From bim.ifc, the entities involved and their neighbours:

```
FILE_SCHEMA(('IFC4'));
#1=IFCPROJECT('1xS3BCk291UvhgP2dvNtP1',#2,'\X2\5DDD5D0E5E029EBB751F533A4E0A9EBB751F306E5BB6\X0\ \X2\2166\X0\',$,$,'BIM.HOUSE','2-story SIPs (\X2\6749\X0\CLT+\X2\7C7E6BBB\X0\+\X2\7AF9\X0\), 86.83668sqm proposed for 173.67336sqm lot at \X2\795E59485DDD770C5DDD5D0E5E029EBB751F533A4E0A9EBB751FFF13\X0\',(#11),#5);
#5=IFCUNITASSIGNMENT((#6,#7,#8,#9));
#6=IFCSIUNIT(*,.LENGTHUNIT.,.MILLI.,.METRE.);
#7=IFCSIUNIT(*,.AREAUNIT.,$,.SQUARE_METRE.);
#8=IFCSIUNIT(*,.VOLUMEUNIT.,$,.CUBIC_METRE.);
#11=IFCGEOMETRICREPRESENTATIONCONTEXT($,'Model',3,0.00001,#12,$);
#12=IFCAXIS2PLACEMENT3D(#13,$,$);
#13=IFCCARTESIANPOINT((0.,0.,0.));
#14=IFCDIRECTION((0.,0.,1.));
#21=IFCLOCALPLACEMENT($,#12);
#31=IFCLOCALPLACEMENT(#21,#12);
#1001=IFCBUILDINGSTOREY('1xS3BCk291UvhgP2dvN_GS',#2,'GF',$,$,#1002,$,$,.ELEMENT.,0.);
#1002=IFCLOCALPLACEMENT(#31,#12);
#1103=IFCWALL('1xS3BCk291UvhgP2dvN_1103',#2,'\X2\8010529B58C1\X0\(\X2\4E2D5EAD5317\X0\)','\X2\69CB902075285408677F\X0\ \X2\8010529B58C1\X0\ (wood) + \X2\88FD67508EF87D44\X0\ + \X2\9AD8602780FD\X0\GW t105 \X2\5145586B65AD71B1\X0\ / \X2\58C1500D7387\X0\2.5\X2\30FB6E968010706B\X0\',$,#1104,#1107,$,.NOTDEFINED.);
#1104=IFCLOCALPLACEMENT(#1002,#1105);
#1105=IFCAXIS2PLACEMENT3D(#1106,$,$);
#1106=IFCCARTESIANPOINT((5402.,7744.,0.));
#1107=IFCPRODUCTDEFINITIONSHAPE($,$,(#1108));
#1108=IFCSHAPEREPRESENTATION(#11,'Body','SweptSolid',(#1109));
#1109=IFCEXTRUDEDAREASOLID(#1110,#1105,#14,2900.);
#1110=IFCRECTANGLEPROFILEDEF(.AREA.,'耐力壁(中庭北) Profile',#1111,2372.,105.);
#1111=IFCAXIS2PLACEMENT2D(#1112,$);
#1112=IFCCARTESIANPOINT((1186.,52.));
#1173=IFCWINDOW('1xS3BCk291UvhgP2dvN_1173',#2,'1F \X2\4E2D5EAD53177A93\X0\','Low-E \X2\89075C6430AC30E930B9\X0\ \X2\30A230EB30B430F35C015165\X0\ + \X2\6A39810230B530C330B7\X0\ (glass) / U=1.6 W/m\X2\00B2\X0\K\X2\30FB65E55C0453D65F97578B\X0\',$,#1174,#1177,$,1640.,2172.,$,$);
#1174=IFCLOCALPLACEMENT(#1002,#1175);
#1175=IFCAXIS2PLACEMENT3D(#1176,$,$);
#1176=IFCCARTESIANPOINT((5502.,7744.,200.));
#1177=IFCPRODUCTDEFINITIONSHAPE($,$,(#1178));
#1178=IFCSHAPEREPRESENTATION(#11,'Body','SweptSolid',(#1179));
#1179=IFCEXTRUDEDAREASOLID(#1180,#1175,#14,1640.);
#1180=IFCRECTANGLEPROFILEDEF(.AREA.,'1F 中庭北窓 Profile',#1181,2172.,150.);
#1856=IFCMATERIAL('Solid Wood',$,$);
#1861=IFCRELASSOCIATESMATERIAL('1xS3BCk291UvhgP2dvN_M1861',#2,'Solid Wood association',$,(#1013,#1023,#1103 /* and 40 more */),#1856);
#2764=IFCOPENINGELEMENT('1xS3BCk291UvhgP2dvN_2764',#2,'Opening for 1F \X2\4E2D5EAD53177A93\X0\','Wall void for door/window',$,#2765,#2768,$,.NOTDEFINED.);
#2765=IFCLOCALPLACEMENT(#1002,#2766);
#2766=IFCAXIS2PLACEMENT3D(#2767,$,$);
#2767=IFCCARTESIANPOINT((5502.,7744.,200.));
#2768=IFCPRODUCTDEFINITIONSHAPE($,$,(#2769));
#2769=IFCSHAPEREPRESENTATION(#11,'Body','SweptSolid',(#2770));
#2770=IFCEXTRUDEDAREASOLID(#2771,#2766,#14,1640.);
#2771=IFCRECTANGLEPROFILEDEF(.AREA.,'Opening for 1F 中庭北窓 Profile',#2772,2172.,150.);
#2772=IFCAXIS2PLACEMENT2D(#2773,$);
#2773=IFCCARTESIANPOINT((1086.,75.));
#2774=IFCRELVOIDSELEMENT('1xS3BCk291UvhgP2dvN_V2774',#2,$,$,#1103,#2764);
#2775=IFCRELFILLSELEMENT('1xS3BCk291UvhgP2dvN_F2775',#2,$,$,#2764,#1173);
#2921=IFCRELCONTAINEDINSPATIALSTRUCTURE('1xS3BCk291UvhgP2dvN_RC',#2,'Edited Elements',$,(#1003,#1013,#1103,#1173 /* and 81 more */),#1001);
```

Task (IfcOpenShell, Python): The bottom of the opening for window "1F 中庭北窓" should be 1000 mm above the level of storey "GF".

```python
import numpy as np
import ifcopenshell
import ifcopenshell.api.geometry
import ifcopenshell.geom
import ifcopenshell.util.element
import ifcopenshell.util.placement
import ifcopenshell.util.shape
import ifcopenshell.util.unit

model = ifcopenshell.open("bim.ifc")
unit_scale = ifcopenshell.util.unit.calculate_unit_scale(model)

window = model.by_guid("1xS3BCk291UvhgP2dvN_1173")
opening = window.FillsVoids[0].RelatingOpeningElement
storey = ifcopenshell.util.element.get_container(window, ifc_class="IfcBuildingStorey")
level = ifcopenshell.util.placement.get_local_placement(storey.ObjectPlacement)[2, 3]

# The opening's origin need not be at the sill, so measure its lowest point.
shape = ifcopenshell.geom.create_shape(ifcopenshell.geom.settings(), opening)
bottom = ifcopenshell.util.shape.get_shape_bottom_elevation(shape, shape.geometry) / unit_scale
dz = level + 1 / unit_scale - bottom

shift = np.array([0.0, 0.0, dz])
# The window is not placed relative to its opening, so move both.
for product in (opening, window):
    matrix = ifcopenshell.util.placement.get_local_placement(product.ObjectPlacement)
    matrix[:3, 3] += shift
    ifcopenshell.api.geometry.edit_object_placement(model, product=product, matrix=matrix, is_si=False)

print(f"moved by {dz * unit_scale:+.3f} m")

model.write("bim_rev.ifc")
```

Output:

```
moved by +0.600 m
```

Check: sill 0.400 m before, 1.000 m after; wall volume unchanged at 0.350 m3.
